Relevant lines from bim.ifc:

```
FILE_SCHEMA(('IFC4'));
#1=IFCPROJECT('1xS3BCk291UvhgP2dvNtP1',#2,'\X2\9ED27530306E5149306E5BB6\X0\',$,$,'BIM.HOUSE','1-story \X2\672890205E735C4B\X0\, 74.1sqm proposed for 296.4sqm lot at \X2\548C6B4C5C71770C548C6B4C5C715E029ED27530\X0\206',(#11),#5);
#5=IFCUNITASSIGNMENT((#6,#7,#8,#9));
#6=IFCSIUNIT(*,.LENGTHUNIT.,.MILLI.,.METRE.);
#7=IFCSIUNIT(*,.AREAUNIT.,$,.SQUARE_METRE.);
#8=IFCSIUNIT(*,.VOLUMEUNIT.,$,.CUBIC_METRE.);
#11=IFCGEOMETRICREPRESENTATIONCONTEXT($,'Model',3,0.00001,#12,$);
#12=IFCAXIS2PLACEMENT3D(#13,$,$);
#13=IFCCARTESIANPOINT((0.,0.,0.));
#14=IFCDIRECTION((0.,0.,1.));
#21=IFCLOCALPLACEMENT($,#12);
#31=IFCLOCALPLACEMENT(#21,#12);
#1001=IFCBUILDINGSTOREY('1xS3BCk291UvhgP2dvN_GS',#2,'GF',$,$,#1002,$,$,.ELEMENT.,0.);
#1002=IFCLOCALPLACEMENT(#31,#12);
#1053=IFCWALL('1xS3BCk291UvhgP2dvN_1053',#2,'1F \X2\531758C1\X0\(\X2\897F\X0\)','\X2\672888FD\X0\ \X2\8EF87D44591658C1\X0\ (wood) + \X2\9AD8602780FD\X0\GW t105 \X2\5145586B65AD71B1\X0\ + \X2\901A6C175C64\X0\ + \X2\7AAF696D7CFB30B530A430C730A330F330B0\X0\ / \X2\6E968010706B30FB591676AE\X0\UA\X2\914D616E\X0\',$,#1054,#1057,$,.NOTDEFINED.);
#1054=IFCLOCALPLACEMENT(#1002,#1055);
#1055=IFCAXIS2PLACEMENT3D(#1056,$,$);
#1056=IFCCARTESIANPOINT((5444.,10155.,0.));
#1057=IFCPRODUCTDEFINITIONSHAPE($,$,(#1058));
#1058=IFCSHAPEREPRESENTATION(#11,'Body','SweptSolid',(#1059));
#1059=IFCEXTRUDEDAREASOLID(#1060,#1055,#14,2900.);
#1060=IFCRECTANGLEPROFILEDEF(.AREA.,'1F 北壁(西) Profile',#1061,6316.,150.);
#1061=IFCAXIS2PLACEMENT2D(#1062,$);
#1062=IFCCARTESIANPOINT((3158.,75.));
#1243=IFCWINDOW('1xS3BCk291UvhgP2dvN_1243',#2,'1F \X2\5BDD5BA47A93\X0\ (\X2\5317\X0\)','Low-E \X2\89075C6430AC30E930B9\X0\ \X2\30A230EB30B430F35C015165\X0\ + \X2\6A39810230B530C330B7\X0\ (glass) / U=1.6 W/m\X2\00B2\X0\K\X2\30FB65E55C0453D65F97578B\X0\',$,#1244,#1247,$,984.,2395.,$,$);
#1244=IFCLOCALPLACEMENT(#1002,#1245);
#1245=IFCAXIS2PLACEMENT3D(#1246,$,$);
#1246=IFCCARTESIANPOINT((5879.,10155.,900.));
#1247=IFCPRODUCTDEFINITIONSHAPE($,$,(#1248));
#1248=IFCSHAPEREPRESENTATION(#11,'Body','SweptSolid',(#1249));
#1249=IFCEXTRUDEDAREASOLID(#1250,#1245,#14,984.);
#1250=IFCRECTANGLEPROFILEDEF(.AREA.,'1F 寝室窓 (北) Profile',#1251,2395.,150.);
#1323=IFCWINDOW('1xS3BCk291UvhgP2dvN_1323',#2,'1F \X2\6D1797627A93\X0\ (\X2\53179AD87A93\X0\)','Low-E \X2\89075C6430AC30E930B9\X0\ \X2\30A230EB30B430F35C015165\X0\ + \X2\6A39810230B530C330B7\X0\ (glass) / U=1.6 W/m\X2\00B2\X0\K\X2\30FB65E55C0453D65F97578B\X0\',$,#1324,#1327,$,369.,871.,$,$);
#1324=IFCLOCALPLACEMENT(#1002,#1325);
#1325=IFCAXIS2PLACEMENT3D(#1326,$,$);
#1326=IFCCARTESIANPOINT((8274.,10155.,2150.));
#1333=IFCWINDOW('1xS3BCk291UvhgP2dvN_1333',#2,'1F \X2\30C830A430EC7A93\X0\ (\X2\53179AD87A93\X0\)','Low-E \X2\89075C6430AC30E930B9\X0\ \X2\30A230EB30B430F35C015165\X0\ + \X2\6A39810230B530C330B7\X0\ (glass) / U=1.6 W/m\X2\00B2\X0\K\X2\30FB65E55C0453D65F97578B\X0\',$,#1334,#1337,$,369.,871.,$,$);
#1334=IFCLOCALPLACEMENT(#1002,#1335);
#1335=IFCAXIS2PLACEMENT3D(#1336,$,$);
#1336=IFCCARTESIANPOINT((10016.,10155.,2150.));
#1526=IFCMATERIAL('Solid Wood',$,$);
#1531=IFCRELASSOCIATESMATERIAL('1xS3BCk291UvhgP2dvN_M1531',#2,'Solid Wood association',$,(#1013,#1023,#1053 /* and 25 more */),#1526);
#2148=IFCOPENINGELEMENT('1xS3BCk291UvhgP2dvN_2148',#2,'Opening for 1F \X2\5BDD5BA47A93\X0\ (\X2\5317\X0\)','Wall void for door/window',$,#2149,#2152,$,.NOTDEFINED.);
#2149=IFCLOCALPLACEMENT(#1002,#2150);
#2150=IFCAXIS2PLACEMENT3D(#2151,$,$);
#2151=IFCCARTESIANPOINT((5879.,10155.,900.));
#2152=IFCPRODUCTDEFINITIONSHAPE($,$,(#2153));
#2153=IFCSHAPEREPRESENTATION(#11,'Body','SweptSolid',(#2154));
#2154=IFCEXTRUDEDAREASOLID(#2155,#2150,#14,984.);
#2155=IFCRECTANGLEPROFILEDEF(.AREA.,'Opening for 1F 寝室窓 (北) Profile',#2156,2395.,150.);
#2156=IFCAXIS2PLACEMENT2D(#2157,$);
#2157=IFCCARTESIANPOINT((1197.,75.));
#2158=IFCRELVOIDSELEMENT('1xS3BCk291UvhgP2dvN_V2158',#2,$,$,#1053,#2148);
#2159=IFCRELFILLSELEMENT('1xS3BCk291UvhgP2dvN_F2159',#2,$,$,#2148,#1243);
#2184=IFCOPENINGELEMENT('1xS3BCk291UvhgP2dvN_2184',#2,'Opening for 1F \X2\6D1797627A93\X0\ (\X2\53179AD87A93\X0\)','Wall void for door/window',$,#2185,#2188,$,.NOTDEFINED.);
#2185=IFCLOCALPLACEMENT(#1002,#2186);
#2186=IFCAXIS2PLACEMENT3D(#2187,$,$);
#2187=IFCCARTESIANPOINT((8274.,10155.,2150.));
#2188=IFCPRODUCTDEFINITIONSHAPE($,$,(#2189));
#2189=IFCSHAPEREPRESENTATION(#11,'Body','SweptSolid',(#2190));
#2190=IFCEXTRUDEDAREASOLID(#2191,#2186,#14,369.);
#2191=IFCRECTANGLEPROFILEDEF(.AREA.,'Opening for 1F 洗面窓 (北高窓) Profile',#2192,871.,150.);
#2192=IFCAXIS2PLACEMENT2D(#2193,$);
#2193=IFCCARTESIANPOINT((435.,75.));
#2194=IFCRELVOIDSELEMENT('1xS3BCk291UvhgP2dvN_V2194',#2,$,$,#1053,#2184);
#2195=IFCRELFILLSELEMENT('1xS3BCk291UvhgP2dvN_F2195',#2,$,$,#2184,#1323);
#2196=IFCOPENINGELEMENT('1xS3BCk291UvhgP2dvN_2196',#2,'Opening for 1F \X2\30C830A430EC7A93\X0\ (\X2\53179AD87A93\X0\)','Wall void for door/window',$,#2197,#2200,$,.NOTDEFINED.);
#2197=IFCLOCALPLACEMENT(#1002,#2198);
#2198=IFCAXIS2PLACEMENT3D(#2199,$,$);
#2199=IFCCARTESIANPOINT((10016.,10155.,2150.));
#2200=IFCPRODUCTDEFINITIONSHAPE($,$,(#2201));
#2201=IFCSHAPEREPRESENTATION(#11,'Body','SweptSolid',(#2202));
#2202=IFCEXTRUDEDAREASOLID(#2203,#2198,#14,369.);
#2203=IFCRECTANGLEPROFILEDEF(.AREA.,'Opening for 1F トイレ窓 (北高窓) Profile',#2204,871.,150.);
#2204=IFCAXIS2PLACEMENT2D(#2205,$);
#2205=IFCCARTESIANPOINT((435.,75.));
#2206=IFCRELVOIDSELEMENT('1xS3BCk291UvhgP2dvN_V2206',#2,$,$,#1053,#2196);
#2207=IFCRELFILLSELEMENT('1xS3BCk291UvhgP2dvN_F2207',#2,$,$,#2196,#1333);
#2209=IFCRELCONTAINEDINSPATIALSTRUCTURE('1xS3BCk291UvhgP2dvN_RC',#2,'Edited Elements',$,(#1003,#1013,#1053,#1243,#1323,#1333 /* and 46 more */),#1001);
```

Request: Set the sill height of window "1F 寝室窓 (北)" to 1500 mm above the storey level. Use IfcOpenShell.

```python
import numpy as np
import ifcopenshell
import ifcopenshell.api.geometry
import ifcopenshell.geom
import ifcopenshell.util.element
import ifcopenshell.util.placement
import ifcopenshell.util.shape
import ifcopenshell.util.unit

model = ifcopenshell.open("bim.ifc")
unit_scale = ifcopenshell.util.unit.calculate_unit_scale(model)

window = model.by_guid("1xS3BCk291UvhgP2dvN_1243")
opening = window.FillsVoids[0].RelatingOpeningElement
storey = ifcopenshell.util.element.get_container(window, ifc_class="IfcBuildingStorey")
level = ifcopenshell.util.placement.get_local_placement(storey.ObjectPlacement)[2, 3]

# The opening's origin need not be at the sill, so measure its lowest point.
shape = ifcopenshell.geom.create_shape(ifcopenshell.geom.settings(), opening)
bottom = ifcopenshell.util.shape.get_shape_bottom_elevation(shape, shape.geometry) / unit_scale
dz = level + 1.5 / unit_scale - bottom

shift = np.array([0.0, 0.0, dz])
# The window is not placed relative to its opening, so move both.
for product in (opening, window):
    matrix = ifcopenshell.util.placement.get_local_placement(product.ObjectPlacement)
    matrix[:3, 3] += shift
    ifcopenshell.api.geometry.edit_object_placement(model, product=product, matrix=matrix, is_si=False)

print(f"moved by {dz * unit_scale:+.3f} m")

model.write("bim_rev.ifc")
```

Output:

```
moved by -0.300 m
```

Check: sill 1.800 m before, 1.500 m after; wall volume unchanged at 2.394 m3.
